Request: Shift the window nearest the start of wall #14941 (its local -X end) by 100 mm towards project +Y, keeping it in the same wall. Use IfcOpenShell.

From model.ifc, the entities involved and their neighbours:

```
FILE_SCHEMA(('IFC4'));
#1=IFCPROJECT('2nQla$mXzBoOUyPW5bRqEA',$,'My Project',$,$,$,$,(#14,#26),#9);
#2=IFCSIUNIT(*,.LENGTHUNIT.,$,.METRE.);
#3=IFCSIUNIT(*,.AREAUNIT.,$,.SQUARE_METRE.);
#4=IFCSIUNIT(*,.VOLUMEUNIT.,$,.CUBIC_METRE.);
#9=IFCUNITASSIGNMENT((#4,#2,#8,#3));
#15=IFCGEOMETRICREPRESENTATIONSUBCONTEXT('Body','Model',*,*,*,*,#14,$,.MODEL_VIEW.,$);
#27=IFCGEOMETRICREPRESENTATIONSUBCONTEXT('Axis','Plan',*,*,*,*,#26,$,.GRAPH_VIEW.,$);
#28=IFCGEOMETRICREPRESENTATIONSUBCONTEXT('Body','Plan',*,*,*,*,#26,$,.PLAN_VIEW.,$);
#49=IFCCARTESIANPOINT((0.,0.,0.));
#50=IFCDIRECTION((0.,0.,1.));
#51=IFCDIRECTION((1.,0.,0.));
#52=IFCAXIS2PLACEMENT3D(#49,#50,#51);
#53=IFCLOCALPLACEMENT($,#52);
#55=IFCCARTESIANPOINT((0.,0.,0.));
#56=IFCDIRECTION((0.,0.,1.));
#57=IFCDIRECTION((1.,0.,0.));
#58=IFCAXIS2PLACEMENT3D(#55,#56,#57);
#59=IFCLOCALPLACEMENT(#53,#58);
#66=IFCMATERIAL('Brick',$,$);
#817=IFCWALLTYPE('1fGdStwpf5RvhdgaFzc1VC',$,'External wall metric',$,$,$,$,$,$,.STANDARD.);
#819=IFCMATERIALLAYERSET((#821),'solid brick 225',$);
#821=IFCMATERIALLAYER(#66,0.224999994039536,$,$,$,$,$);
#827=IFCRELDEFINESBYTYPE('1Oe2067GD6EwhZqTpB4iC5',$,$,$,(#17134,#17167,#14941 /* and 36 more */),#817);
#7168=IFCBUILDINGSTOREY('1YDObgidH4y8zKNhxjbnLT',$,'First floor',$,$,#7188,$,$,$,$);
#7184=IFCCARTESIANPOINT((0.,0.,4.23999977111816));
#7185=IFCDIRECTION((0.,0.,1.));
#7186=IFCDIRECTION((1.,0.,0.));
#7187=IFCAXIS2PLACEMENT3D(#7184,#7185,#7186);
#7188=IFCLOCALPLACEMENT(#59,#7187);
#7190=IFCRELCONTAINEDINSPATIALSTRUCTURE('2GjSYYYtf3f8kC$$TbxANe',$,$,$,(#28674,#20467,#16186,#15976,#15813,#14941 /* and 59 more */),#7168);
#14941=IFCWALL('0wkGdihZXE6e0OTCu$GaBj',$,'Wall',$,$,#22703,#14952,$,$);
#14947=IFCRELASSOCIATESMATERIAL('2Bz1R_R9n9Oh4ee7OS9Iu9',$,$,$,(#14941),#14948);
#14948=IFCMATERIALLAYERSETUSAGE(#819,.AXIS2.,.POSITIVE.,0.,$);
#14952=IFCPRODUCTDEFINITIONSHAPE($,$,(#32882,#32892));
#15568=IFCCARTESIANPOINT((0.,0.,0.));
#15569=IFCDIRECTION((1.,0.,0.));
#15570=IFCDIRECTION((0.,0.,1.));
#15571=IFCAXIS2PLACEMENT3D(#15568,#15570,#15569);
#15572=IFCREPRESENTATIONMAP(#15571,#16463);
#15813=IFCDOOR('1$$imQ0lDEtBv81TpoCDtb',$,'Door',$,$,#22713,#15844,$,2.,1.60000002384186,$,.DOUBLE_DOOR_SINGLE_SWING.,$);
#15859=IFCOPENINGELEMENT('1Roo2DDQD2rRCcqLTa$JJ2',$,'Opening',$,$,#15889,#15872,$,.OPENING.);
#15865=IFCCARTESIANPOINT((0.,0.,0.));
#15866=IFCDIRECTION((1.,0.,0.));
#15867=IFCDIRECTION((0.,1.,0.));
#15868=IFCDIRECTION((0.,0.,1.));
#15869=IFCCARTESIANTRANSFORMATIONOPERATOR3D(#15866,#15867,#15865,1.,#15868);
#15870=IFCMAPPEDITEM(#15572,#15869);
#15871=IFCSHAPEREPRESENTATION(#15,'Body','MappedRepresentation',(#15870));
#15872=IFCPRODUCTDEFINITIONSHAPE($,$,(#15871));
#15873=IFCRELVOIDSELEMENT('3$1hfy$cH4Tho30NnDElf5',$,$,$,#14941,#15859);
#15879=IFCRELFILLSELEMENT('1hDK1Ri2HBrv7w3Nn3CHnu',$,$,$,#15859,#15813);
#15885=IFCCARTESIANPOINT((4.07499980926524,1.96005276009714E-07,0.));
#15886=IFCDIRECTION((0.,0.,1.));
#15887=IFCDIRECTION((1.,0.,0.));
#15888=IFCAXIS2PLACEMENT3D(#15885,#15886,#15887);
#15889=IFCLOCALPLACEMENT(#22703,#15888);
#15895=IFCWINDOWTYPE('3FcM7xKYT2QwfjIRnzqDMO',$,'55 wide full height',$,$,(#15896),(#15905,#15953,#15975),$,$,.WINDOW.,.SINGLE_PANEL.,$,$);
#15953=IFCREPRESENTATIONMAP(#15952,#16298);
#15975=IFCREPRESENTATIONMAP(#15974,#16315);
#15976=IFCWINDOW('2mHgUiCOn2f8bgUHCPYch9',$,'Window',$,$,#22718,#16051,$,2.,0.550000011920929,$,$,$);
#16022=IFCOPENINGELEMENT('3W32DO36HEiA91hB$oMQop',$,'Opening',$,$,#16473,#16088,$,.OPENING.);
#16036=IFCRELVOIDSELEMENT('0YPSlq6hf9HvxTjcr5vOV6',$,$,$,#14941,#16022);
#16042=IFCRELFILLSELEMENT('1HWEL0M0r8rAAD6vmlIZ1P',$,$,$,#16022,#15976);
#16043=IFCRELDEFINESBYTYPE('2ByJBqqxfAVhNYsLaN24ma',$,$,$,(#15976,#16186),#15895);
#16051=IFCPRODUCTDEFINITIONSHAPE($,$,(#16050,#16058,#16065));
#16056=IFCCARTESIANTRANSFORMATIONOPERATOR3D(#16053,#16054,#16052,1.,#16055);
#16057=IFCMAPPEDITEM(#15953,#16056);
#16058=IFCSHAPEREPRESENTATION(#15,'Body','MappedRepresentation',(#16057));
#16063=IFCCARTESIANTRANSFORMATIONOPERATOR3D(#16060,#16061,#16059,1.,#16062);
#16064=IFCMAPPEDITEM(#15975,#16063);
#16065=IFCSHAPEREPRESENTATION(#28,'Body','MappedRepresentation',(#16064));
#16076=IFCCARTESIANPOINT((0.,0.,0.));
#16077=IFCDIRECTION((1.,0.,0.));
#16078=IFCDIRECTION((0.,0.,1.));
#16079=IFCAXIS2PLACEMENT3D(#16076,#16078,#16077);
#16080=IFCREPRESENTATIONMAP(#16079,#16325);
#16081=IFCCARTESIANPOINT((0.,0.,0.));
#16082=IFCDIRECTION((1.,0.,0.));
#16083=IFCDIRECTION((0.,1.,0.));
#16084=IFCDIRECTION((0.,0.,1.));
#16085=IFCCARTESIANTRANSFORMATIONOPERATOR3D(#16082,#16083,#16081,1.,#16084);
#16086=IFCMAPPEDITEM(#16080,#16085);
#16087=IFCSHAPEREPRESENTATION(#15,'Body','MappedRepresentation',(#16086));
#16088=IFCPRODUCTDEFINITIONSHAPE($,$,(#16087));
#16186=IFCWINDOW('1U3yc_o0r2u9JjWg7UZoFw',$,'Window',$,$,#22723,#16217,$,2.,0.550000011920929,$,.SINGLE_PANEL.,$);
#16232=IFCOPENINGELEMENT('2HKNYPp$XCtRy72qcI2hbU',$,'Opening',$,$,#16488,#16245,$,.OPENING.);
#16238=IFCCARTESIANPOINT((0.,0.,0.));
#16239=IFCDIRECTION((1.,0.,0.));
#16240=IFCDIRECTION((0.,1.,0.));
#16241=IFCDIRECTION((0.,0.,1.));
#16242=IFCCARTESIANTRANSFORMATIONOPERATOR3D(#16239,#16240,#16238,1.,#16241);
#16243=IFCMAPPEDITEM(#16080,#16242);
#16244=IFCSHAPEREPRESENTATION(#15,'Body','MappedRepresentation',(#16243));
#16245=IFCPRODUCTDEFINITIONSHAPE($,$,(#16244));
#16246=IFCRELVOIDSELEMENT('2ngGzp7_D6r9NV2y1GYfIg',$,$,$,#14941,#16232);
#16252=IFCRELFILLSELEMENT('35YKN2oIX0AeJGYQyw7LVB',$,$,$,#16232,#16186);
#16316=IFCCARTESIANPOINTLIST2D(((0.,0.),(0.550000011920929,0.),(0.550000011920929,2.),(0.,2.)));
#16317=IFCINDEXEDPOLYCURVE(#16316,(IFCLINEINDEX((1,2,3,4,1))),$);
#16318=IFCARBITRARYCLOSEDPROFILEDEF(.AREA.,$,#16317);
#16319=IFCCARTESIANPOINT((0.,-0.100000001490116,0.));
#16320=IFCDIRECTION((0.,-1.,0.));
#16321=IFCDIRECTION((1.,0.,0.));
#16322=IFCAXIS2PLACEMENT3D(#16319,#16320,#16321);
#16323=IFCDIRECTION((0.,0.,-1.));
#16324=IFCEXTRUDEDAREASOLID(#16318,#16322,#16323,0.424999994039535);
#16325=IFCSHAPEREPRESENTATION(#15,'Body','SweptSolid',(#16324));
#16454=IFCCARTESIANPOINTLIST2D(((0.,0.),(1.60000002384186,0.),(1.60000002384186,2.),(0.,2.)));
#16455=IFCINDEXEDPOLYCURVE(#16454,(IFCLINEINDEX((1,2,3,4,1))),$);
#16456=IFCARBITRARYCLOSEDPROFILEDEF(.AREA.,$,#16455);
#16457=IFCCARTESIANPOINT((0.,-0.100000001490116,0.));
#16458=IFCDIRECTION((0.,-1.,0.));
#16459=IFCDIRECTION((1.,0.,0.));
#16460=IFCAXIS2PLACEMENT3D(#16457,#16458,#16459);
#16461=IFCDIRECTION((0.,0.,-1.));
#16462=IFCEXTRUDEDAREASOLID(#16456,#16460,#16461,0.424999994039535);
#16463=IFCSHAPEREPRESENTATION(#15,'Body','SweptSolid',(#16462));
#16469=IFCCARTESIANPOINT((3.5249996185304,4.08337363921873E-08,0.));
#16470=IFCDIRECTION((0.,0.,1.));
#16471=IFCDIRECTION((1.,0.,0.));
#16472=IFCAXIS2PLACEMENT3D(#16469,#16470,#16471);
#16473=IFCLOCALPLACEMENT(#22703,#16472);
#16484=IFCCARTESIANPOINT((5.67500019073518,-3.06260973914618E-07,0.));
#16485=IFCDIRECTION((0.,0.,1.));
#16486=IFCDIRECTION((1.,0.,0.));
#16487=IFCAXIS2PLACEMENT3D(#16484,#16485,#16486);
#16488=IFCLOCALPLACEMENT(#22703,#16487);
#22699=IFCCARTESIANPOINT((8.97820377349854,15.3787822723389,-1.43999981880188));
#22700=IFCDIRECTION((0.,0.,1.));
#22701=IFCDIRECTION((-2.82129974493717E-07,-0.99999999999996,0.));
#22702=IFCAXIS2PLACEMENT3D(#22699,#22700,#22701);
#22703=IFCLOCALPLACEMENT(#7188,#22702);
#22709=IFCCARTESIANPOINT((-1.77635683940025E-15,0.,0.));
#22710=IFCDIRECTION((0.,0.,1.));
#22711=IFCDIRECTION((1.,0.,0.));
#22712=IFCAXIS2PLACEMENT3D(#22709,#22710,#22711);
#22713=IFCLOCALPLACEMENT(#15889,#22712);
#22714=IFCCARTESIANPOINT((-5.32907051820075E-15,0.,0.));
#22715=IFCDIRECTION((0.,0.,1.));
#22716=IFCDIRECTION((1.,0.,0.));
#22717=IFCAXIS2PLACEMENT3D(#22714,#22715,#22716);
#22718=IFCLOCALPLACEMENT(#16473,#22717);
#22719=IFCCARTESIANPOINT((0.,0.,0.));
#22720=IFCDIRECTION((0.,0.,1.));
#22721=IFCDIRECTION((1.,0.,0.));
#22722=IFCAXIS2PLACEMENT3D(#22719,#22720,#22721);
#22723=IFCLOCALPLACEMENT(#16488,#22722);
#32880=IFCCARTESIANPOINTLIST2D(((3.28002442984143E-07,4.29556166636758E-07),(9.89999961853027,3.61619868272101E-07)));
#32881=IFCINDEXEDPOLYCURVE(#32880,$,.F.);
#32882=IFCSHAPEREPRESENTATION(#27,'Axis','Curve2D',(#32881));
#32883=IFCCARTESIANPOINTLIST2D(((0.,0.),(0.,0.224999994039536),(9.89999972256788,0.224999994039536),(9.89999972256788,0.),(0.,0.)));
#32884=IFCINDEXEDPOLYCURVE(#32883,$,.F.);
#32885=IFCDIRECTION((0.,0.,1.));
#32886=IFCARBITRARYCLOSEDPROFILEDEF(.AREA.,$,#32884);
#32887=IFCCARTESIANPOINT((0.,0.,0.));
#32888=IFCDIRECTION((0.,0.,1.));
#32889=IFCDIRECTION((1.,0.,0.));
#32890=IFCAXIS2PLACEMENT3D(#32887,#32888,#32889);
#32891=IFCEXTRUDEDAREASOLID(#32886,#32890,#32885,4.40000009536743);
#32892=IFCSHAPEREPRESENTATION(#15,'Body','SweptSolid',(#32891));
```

```python
import ifcopenshell
import ifcopenshell.api.geometry
import ifcopenshell.util.placement

model = ifcopenshell.open("model.ifc")

window = model.by_id(15976)
opening = window.FillsVoids[0].RelatingOpeningElement
wall = opening.VoidsElements[0].RelatingBuildingElement

wall_matrix = ifcopenshell.util.placement.get_local_placement(wall.ObjectPlacement)
shift = wall_matrix[:3, 0] * -0.1
before = ifcopenshell.util.placement.get_local_placement(window.ObjectPlacement)[:3, 3].copy()

# The window is placed relative to its opening, so it follows when the opening moves.
matrix = ifcopenshell.util.placement.get_local_placement(opening.ObjectPlacement)
matrix[:3, 3] += shift
ifcopenshell.api.geometry.edit_object_placement(
    model, product=opening, matrix=matrix, is_si=False, should_transform_children=True
)

after = ifcopenshell.util.placement.get_local_placement(window.ObjectPlacement)[:3, 3]
print("window moved by", (after - before).round(3) + 0.0)

model.write("model_updated.ifc")
```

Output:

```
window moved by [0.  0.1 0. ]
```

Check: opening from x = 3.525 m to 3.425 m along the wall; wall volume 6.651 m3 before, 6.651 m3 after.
